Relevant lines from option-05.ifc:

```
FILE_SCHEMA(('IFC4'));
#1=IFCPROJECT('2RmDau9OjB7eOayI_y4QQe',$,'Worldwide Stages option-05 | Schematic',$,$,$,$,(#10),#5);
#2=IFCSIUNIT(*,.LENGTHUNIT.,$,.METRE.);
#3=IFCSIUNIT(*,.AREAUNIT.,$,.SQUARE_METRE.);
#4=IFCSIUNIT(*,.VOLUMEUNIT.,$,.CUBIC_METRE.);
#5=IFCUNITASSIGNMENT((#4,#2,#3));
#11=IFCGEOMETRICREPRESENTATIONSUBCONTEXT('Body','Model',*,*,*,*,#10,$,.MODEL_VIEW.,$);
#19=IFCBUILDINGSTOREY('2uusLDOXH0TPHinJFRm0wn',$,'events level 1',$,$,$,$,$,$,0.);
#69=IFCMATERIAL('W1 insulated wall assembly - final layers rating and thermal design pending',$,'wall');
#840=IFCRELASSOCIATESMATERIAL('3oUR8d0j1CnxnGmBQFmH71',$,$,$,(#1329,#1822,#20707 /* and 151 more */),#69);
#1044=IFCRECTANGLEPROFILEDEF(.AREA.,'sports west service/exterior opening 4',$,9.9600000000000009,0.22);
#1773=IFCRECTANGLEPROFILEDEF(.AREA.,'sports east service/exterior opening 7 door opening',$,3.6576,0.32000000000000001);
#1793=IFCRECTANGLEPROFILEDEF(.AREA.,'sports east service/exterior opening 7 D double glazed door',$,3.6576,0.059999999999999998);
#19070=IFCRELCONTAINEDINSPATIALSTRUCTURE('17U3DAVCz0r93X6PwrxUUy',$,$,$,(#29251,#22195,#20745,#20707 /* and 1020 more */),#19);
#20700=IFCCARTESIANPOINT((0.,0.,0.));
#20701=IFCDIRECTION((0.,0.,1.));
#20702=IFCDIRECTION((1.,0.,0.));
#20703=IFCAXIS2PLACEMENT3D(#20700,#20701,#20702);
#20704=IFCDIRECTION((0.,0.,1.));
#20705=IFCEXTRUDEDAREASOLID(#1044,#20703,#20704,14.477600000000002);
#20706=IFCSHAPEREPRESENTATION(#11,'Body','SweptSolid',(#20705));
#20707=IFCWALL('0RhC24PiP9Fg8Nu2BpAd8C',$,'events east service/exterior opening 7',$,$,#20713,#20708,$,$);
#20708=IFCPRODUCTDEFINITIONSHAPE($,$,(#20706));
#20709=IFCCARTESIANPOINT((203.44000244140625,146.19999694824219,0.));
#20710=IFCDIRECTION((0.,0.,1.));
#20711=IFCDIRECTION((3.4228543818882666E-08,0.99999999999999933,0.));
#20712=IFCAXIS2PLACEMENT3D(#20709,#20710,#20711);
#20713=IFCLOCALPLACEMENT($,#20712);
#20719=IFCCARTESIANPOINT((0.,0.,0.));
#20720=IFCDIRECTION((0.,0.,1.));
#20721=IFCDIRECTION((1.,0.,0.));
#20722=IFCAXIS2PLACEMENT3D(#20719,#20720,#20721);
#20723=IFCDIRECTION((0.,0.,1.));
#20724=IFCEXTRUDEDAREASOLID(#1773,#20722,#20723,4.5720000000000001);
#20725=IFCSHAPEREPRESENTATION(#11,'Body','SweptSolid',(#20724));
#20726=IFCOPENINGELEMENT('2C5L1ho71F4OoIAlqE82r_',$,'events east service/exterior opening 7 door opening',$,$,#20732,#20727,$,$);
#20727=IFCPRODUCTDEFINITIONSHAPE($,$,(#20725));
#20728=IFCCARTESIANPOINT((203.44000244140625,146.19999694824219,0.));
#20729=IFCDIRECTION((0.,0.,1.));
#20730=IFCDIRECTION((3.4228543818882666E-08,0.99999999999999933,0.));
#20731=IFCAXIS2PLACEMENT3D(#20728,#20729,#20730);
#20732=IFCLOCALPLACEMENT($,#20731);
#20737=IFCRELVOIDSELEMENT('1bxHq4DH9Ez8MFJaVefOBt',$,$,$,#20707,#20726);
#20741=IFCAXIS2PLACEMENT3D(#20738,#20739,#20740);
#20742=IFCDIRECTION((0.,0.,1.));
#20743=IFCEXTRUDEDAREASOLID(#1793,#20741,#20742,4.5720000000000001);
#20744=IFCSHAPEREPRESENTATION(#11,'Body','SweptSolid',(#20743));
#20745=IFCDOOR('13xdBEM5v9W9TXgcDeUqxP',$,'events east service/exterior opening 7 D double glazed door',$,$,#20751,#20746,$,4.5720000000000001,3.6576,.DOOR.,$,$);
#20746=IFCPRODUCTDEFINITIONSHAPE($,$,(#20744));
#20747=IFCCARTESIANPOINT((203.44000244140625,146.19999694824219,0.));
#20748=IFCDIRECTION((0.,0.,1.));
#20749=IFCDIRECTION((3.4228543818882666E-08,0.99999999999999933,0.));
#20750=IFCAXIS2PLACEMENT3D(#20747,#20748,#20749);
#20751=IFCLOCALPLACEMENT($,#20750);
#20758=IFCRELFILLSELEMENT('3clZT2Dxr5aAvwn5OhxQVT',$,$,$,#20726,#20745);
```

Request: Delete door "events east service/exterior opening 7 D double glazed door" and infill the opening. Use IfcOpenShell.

```python
import ifcopenshell
import ifcopenshell.api.feature
import ifcopenshell.api.root
import ifcopenshell.geom
import ifcopenshell.util.shape

model = ifcopenshell.open("option-05.ifc")
settings = ifcopenshell.geom.settings()


def volume(element):
    """Net volume in cubic metres, openings subtracted."""
    shape = ifcopenshell.geom.create_shape(settings, element)
    return ifcopenshell.util.shape.get_volume(shape.geometry)


door = model.by_guid("13xdBEM5v9W9TXgcDeUqxP")
opening = door.FillsVoids[0].RelatingOpeningElement
wall = opening.VoidsElements[0].RelatingBuildingElement
before = volume(wall)

ifcopenshell.api.root.remove_product(model, product=door)
ifcopenshell.api.feature.remove_feature(model, feature=opening)

after = volume(wall)

print(f"wall volume {before:.3f} -> {after:.3f} m3")

model.write("option-05_rev.ifc")
```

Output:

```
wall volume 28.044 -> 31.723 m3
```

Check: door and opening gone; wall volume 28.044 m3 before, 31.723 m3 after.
